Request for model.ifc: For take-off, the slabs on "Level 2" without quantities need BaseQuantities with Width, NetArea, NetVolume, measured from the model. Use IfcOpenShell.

First a look at what the model holds.

```python
import ifcopenshell
import ifcopenshell.util.element
import ifcopenshell.util.unit

model = ifcopenshell.open("model.ifc")
print(model.schema)
for unit_type in ("LENGTHUNIT", "AREAUNIT", "VOLUMEUNIT"):
    print(unit_type, ifcopenshell.util.unit.calculate_unit_scale(model, unit_type))
storey = next(s for s in model.by_type("IfcBuildingStorey") if s.Name == "Level 2")
slabs = [e for e in ifcopenshell.util.element.get_decomposition(storey) if e.is_a("IfcSlab")]
for e in sorted(slabs, key=lambda e: e.id()):
    print(e.id(), e.is_a(), e.Name, list(ifcopenshell.util.element.get_psets(e, qtos_only=True)), sep=" | ")
```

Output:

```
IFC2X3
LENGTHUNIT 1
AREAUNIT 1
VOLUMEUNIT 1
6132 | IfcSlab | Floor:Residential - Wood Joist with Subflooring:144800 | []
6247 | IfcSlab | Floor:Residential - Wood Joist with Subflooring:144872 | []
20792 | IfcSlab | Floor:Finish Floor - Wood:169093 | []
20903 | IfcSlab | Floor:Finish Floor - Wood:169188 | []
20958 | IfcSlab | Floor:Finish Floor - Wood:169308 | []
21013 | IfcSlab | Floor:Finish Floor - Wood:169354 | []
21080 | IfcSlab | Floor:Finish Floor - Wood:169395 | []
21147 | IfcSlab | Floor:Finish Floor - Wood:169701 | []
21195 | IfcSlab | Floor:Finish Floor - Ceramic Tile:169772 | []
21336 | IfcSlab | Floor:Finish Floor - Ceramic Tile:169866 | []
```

```python
import ifcopenshell
import ifcopenshell.api.pset
import ifcopenshell.geom
import ifcopenshell.util.element
import ifcopenshell.util.shape
import ifcopenshell.util.unit

model = ifcopenshell.open("model.ifc")
unit_scale = ifcopenshell.util.unit.calculate_unit_scale(model)
area_scale = ifcopenshell.util.unit.calculate_unit_scale(model, "AREAUNIT")
volume_scale = ifcopenshell.util.unit.calculate_unit_scale(model, "VOLUMEUNIT")
settings = ifcopenshell.geom.settings()

storey = next(s for s in model.by_type("IfcBuildingStorey") if s.Name == "Level 2")
slabs = [e for e in ifcopenshell.util.element.get_decomposition(storey) if e.is_a("IfcSlab")]

for e in sorted(slabs, key=lambda e: e.id()):
    if ifcopenshell.util.element.get_psets(e, qtos_only=True, should_inherit=False):
        continue
    # Geometry comes back in metres, in the element's own axes.
    shape = ifcopenshell.geom.create_shape(settings, e)
    values = {
        "Width": ifcopenshell.util.shape.get_z(shape.geometry) / unit_scale,
        "NetArea": ifcopenshell.util.shape.get_footprint_area(shape.geometry) / area_scale,
        "NetVolume": ifcopenshell.util.shape.get_volume(shape.geometry) / volume_scale,
    }
    qto = ifcopenshell.api.pset.add_qto(model, product=e, name="BaseQuantities")
    ifcopenshell.api.pset.edit_qto(model, qto=qto, properties=values)
    print(e.id(), {k: round(v, 3) for k, v in values.items()})

model.write("model_v2.ifc")
```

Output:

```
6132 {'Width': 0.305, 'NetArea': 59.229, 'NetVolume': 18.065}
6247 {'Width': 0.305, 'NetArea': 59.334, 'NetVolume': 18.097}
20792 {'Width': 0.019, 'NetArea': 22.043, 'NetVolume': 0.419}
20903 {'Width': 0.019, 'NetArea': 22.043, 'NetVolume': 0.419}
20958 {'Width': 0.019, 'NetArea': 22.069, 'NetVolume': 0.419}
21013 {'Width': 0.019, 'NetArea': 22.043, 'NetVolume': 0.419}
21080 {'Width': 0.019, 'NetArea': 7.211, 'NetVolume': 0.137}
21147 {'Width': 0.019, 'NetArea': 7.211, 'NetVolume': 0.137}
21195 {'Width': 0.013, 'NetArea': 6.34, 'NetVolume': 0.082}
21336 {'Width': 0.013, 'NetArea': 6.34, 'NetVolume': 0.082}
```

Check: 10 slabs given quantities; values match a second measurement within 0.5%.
